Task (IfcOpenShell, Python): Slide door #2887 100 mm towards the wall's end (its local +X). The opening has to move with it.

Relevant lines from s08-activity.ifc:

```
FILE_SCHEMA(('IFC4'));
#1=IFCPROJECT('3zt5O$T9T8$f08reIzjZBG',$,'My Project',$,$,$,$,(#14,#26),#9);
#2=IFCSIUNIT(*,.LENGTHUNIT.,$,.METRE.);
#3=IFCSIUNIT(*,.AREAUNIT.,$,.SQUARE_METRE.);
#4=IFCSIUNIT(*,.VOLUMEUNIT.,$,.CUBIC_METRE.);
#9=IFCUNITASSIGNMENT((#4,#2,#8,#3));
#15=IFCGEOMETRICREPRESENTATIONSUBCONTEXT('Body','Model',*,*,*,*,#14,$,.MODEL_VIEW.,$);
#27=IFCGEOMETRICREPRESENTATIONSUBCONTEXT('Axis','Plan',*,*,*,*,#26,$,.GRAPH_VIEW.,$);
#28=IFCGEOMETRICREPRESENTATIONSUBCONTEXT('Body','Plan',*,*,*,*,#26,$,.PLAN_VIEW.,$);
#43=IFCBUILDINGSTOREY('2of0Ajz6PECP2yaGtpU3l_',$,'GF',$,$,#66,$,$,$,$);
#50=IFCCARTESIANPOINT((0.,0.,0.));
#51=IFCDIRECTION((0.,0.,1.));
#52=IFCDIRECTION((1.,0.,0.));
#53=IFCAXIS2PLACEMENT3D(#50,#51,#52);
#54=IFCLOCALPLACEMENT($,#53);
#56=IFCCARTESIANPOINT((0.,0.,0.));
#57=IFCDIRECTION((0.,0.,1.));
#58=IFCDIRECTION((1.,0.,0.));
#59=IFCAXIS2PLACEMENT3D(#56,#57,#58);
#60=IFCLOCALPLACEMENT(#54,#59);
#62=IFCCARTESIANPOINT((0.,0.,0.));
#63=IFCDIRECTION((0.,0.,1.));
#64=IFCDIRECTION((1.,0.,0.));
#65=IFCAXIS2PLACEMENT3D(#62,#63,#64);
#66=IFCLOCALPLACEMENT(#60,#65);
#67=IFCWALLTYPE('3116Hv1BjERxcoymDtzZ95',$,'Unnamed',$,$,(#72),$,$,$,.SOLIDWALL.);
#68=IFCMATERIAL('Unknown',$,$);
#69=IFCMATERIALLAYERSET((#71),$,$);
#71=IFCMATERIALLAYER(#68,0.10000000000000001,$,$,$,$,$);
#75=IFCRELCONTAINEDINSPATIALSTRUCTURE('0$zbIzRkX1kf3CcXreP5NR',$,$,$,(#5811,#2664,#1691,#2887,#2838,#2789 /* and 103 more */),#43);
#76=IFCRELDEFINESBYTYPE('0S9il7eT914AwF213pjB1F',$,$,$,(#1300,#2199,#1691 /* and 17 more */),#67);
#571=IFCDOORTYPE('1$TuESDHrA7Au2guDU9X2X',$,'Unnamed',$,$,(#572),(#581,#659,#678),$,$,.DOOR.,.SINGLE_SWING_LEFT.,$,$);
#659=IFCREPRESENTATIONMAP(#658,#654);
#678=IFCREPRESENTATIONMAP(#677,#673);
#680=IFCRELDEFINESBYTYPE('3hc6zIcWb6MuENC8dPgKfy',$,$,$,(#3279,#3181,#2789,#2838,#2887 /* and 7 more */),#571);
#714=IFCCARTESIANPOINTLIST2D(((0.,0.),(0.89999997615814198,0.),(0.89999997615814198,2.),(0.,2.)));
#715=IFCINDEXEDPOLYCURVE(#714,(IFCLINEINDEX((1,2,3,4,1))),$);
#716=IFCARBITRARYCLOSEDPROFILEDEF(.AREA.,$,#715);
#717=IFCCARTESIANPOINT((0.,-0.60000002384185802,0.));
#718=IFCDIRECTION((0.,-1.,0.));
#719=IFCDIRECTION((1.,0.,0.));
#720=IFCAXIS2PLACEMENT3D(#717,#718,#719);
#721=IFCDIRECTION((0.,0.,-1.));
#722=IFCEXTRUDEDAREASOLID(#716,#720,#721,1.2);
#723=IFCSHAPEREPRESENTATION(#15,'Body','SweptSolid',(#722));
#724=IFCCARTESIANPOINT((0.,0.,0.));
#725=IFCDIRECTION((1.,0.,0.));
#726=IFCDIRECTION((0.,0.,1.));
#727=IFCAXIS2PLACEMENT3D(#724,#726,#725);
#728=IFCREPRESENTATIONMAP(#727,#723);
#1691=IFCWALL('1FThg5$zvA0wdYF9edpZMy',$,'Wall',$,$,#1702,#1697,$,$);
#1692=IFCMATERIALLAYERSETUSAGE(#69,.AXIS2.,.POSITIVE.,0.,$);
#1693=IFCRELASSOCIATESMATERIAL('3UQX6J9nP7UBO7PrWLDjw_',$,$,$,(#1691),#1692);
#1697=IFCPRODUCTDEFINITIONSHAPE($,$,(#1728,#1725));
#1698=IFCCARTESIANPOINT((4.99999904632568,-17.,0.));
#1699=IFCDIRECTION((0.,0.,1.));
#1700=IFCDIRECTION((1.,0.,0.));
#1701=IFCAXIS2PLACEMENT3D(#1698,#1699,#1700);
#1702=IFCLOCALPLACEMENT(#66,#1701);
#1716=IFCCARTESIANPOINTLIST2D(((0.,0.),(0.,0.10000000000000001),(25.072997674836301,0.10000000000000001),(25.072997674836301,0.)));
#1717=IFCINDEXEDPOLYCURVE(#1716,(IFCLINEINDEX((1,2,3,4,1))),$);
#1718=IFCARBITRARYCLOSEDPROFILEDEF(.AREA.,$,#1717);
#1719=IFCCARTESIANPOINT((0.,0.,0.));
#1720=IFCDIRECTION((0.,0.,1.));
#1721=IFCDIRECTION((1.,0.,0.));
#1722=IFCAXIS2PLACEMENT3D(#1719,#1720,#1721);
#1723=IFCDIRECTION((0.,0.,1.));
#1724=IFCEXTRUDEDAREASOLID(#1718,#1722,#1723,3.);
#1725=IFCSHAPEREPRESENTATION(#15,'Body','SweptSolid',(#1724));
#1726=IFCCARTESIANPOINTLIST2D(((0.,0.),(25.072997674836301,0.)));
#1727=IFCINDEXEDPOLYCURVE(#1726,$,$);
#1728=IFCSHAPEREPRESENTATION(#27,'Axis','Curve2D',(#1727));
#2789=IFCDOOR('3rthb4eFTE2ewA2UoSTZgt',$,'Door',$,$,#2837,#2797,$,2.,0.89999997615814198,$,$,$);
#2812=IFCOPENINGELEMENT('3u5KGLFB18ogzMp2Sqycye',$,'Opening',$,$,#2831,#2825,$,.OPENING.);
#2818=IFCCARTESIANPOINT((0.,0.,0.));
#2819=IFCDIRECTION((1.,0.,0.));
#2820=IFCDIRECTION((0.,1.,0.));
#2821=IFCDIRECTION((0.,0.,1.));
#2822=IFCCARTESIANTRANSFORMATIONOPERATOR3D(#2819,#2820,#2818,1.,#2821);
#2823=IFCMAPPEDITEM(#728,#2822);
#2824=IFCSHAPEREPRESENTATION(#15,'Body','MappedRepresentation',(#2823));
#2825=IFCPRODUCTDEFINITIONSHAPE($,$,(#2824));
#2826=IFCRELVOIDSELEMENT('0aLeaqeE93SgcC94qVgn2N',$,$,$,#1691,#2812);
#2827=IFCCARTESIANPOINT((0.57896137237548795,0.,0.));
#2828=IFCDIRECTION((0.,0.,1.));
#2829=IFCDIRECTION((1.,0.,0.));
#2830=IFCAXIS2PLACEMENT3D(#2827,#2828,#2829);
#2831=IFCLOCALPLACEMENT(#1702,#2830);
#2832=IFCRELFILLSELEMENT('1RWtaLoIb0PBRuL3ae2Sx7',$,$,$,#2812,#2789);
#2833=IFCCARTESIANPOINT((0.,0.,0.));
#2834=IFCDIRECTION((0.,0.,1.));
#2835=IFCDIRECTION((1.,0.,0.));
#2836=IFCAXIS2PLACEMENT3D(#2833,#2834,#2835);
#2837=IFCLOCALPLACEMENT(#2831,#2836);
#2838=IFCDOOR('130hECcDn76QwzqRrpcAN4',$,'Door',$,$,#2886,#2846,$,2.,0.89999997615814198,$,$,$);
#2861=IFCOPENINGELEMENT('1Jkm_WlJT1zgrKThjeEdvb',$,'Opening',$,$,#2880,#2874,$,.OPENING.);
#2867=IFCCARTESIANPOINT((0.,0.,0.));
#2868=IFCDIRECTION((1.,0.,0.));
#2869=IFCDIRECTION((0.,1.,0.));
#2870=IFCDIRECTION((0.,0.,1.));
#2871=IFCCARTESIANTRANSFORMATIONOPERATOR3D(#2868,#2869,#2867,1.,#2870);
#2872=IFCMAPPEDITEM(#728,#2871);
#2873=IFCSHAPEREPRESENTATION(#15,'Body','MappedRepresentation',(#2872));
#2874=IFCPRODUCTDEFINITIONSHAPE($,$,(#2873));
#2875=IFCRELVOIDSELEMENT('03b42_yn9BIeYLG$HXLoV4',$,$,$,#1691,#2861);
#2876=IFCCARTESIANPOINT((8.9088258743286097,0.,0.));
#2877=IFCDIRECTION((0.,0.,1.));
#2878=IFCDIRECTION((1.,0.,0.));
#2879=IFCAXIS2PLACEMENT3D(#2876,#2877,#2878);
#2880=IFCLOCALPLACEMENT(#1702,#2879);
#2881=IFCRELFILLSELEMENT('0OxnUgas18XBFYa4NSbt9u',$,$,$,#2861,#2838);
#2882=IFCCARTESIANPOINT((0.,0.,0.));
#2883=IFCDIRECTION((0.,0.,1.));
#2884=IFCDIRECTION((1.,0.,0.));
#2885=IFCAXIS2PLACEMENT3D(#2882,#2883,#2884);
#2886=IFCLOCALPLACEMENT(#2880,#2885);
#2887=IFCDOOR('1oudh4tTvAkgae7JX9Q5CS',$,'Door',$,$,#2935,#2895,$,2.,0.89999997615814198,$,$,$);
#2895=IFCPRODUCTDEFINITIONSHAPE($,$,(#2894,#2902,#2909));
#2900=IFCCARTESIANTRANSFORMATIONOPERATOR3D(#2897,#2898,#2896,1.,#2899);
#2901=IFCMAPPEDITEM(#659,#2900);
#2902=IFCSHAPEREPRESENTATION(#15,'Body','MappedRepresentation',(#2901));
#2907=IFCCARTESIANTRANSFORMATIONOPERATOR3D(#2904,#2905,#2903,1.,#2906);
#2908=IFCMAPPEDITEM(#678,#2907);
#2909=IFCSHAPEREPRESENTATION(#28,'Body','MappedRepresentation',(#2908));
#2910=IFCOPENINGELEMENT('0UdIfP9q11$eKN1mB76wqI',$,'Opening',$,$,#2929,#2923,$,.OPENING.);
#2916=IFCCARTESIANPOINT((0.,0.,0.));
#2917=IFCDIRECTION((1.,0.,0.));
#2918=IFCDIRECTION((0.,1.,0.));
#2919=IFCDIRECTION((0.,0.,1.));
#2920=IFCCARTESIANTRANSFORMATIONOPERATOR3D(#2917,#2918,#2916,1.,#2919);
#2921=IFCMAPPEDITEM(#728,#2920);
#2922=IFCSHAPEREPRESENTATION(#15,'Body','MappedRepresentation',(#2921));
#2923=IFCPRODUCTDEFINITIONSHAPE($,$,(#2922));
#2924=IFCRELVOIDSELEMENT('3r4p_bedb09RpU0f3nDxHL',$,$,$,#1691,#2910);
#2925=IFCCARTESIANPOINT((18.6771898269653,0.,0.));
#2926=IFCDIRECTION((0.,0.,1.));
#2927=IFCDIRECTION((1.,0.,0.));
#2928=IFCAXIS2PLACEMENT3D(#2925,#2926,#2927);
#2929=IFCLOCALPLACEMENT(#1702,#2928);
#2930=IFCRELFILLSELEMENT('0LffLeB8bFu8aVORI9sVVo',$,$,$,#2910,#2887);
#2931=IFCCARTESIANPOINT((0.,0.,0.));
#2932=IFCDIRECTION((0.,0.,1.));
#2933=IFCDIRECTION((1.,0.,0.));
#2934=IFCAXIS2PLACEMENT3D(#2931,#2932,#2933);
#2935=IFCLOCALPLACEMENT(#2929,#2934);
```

```python
import ifcopenshell
import ifcopenshell.api.geometry
import ifcopenshell.util.placement
import ifcopenshell.util.unit

model = ifcopenshell.open("s08-activity.ifc")
unit_scale = ifcopenshell.util.unit.calculate_unit_scale(model)

door = model.by_guid("1oudh4tTvAkgae7JX9Q5CS")
opening = door.FillsVoids[0].RelatingOpeningElement
wall = opening.VoidsElements[0].RelatingBuildingElement

wall_matrix = ifcopenshell.util.placement.get_local_placement(wall.ObjectPlacement)
shift = wall_matrix[:3, 0] * 0.1 / unit_scale
before = ifcopenshell.util.placement.get_local_placement(door.ObjectPlacement)[:3, 3].copy()

# The door is placed relative to its opening, so it follows when the opening moves.
matrix = ifcopenshell.util.placement.get_local_placement(opening.ObjectPlacement)
matrix[:3, 3] += shift
ifcopenshell.api.geometry.edit_object_placement(
    model, product=opening, matrix=matrix, is_si=False, should_transform_children=True
)

after = ifcopenshell.util.placement.get_local_placement(door.ObjectPlacement)[:3, 3]
print("door moved by", (after - before).round(3) + 0.0)

model.write("s08-activity_rev.ifc")
```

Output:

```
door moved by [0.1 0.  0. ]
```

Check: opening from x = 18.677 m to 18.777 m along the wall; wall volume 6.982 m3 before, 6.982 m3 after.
